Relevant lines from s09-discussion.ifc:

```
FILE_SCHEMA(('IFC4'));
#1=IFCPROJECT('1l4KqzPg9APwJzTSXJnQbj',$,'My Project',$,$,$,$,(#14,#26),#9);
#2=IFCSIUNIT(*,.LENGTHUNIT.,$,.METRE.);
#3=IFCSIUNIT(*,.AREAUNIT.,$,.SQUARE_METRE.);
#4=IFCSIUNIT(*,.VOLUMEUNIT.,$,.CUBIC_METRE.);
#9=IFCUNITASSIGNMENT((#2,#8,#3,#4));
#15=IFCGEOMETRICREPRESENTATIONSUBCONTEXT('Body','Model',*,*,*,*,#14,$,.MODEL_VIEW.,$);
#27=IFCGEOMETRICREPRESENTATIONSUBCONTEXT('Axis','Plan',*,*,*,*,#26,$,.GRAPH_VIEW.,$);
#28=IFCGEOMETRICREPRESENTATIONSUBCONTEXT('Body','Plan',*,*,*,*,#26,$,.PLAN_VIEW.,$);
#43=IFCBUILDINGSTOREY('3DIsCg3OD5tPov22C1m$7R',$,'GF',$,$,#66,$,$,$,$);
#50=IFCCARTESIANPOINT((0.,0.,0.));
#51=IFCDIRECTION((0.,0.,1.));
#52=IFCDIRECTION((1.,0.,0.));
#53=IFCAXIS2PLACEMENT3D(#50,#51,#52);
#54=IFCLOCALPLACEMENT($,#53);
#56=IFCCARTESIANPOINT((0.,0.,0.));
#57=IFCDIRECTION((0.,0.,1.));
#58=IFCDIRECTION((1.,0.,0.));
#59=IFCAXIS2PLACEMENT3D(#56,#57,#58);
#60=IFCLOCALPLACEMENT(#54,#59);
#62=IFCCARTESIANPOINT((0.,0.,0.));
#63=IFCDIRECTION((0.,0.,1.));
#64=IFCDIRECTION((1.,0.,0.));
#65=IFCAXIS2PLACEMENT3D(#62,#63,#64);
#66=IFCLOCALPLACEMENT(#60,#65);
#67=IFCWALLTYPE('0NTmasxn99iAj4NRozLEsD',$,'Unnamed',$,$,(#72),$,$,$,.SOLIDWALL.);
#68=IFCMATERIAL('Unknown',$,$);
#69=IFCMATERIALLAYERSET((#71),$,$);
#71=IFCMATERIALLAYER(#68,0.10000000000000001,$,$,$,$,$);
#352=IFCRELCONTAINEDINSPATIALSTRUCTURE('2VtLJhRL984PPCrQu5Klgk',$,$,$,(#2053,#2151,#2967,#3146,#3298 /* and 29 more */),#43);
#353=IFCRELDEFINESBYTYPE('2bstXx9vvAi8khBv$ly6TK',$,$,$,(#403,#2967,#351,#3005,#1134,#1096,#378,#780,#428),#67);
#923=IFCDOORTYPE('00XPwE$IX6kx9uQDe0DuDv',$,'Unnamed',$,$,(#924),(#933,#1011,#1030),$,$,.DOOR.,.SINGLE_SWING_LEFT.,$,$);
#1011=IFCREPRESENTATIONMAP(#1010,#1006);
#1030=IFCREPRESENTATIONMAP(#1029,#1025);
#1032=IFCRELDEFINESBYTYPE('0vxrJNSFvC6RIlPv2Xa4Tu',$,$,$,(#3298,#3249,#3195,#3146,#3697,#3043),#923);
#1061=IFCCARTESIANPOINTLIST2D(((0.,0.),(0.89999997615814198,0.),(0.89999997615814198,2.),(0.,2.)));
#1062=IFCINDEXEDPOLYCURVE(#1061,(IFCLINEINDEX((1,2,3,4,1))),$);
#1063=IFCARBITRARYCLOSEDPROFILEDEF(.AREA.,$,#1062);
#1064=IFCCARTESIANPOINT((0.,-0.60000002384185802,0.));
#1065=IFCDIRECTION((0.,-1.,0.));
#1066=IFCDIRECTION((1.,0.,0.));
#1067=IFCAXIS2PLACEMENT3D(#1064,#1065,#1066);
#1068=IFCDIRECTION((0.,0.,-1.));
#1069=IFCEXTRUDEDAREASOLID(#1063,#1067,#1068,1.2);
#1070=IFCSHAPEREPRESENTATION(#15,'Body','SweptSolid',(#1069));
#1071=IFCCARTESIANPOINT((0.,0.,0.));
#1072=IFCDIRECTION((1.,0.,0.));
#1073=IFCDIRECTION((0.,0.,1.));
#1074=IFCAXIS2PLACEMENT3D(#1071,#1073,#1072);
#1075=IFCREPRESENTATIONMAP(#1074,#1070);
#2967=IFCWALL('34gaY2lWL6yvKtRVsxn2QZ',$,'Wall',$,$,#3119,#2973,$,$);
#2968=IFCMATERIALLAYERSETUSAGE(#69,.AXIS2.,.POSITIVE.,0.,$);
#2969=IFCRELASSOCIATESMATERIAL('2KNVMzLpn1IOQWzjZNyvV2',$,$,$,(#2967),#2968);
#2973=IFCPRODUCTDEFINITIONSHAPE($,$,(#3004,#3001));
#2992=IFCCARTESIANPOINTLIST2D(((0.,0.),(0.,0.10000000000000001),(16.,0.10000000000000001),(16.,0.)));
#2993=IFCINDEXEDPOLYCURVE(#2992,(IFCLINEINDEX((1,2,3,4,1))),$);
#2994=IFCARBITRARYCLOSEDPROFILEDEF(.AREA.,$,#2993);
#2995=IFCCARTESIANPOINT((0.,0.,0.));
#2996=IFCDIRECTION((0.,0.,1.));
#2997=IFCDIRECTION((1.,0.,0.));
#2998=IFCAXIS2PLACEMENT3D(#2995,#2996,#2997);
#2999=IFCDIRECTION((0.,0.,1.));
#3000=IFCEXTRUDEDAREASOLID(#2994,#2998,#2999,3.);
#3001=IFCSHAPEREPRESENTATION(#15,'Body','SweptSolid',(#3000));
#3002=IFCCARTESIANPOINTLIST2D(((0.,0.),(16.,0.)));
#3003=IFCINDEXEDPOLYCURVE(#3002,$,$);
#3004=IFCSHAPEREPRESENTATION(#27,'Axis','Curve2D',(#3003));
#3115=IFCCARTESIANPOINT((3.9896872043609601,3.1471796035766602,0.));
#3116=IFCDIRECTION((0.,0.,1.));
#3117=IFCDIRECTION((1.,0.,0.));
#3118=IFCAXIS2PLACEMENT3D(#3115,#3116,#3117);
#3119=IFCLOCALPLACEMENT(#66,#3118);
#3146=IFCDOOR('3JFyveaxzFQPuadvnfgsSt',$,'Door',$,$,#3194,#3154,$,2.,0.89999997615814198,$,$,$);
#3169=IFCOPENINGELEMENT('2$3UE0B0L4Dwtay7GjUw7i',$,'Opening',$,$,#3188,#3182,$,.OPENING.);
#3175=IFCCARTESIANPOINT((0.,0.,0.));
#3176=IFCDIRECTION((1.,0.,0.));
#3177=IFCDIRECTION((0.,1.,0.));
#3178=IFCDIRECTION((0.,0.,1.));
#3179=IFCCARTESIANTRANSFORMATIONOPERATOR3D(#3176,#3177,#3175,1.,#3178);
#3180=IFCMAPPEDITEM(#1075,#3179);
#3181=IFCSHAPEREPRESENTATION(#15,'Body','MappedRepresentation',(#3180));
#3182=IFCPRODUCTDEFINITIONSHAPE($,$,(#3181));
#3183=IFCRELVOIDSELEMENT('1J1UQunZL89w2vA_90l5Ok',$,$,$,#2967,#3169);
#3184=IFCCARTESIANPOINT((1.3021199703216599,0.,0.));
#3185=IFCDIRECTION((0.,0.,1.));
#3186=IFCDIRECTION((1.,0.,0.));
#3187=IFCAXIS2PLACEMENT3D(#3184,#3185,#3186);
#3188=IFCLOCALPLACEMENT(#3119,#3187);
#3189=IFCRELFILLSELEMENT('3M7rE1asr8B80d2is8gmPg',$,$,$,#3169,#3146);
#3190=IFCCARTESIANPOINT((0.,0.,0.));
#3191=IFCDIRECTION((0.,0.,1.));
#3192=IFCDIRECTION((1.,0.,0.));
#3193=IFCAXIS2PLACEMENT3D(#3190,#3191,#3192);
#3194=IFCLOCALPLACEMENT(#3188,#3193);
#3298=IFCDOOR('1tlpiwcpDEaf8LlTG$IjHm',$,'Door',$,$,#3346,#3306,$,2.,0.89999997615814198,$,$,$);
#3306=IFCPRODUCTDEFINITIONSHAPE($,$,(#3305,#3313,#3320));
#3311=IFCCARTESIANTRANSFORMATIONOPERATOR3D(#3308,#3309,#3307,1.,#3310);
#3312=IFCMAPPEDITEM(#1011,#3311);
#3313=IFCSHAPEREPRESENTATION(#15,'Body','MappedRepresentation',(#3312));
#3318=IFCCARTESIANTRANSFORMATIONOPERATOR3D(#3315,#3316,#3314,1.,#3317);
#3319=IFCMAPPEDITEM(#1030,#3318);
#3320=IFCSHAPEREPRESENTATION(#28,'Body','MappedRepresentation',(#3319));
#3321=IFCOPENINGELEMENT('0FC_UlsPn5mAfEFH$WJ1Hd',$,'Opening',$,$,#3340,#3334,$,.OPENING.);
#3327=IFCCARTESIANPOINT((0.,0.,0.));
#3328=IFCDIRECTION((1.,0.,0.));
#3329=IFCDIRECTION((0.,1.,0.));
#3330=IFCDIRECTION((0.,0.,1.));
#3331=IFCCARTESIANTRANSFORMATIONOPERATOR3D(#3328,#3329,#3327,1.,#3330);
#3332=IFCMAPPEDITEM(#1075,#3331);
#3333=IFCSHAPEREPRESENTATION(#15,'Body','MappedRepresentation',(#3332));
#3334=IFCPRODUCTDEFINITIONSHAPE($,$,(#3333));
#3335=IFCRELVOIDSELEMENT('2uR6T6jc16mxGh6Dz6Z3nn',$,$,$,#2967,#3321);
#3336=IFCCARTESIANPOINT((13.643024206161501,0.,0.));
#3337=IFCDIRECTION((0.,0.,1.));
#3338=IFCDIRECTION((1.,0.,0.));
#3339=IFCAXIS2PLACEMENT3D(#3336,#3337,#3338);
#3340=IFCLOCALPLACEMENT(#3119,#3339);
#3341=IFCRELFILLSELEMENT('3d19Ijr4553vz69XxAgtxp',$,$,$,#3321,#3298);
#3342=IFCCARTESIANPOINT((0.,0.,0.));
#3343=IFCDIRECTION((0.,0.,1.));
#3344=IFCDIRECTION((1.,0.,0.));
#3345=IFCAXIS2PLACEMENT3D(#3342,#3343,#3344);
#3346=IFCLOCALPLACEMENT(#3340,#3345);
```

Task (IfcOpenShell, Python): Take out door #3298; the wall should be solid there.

```python
import ifcopenshell
import ifcopenshell.api.feature
import ifcopenshell.api.root
import ifcopenshell.geom
import ifcopenshell.util.shape

model = ifcopenshell.open("s09-discussion.ifc")
settings = ifcopenshell.geom.settings()


def volume(element):
    """Net volume in cubic metres, openings subtracted."""
    shape = ifcopenshell.geom.create_shape(settings, element)
    return ifcopenshell.util.shape.get_volume(shape.geometry)


door = model.by_guid("1tlpiwcpDEaf8LlTG$IjHm")
opening = door.FillsVoids[0].RelatingOpeningElement
wall = opening.VoidsElements[0].RelatingBuildingElement
before = volume(wall)

ifcopenshell.api.root.remove_product(model, product=door)
ifcopenshell.api.feature.remove_feature(model, feature=opening)

after = volume(wall)

print(f"wall volume {before:.3f} -> {after:.3f} m3")

model.write("s09-discussion-out.ifc")
```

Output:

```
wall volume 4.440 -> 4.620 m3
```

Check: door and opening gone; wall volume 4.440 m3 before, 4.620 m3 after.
